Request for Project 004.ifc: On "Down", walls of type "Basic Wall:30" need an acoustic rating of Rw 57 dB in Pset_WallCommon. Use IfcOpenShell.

First a look at what the model holds.

```python
import ifcopenshell
import ifcopenshell.util.element

model = ifcopenshell.open("Project 004.ifc")
print(model.schema)
storey = next(s for s in model.by_type("IfcBuildingStorey") if s.Name == "Down")
walls = [e for e in ifcopenshell.util.element.get_decomposition(storey) if e.is_a("IfcWall")]
seen = {}
for e in walls:
    element_type = ifcopenshell.util.element.get_type(e)
    key = (element_type.Name if element_type != e and element_type else None, ifcopenshell.util.element.get_pset(e, "Pset_WallCommon", "AcousticRating"))
    seen[key] = seen.get(key, 0) + 1
for (name, value), count in sorted(seen.items(), key=str):
    print(count, "x", name, "|", value)
```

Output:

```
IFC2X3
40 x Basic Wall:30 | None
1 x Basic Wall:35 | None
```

```python
import ifcopenshell
import ifcopenshell.api.pset
import ifcopenshell.util.element

model = ifcopenshell.open("Project 004.ifc")

storey = next(s for s in model.by_type("IfcBuildingStorey") if s.Name == "Down")
walls = [e for e in ifcopenshell.util.element.get_decomposition(storey) if e.is_a("IfcWall")]

count = 0
for e in walls:
    element_type = ifcopenshell.util.element.get_type(e)
    if element_type in (None, e) or element_type.Name != "Basic Wall:30":
        continue
    # add_pset returns the element's existing set when there is one.
    pset = ifcopenshell.api.pset.add_pset(model, product=e, name="Pset_WallCommon")
    ifcopenshell.api.pset.edit_pset(model, pset=pset, properties={"AcousticRating": "Rw 57 dB"})
    count += 1

print(count, "walls updated")

model.write("Project 004_edited.ifc")
```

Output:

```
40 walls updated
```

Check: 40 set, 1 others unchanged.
